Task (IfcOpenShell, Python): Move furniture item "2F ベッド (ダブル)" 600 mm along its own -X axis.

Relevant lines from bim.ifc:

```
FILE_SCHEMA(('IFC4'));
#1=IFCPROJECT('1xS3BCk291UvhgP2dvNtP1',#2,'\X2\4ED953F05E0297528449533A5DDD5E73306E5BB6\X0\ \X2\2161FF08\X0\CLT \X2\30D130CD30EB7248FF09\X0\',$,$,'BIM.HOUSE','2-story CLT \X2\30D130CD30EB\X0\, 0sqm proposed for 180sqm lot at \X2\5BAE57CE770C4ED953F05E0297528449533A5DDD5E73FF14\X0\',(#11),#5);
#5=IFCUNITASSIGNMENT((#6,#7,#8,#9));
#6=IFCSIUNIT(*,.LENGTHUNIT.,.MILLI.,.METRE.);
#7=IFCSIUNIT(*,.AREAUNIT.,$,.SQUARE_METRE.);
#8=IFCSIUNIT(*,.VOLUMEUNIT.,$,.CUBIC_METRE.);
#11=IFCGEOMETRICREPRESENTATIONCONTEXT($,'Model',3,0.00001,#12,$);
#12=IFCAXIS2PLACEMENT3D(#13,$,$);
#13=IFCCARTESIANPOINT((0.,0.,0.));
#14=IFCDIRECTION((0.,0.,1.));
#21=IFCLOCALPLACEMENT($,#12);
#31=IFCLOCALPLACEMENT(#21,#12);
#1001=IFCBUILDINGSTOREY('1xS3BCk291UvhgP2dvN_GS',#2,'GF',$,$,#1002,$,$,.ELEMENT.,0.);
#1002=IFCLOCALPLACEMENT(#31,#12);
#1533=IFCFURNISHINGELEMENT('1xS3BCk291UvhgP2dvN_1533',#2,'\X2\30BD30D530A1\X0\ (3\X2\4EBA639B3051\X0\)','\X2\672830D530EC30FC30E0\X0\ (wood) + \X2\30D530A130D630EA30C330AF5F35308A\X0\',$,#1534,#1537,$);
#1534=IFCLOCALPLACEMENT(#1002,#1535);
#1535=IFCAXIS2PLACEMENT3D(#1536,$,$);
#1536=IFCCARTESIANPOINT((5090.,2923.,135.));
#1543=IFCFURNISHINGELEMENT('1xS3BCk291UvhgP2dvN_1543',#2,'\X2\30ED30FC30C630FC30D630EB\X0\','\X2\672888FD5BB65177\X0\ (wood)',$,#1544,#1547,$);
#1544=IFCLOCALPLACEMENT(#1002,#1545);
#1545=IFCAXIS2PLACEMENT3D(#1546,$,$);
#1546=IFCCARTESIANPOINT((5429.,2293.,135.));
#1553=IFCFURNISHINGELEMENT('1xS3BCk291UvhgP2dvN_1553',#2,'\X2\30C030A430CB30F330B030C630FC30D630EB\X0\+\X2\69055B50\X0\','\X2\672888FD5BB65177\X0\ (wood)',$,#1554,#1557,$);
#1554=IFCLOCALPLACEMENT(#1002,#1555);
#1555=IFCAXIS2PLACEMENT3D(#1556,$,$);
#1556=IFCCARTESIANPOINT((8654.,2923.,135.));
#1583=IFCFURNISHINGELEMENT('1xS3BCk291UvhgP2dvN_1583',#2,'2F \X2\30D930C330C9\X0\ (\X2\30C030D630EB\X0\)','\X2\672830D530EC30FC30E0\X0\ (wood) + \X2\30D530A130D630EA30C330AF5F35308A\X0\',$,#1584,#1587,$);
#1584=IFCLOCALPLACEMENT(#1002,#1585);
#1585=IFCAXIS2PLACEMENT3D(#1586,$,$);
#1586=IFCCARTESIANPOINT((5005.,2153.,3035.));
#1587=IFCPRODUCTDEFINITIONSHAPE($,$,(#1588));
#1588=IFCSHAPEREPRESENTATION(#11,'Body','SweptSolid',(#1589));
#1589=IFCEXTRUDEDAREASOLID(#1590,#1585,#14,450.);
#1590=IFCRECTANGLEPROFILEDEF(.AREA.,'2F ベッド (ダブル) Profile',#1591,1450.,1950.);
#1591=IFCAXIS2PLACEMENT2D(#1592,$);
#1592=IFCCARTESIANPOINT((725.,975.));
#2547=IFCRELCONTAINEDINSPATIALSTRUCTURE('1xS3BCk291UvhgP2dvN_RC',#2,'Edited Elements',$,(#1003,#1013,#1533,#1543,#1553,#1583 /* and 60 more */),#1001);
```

```python
import ifcopenshell
import ifcopenshell.api.geometry
import ifcopenshell.util.placement
import ifcopenshell.util.unit

model = ifcopenshell.open("bim.ifc")
unit_scale = ifcopenshell.util.unit.calculate_unit_scale(model)

item = model.by_guid("1xS3BCk291UvhgP2dvN_1583")
matrix = ifcopenshell.util.placement.get_local_placement(item.ObjectPlacement)
matrix[:3, 3] -= matrix[:3, 0] * 0.6 / unit_scale
ifcopenshell.api.geometry.edit_object_placement(model, product=item, matrix=matrix, is_si=False)

print(ifcopenshell.util.placement.get_local_placement(item.ObjectPlacement).round(3) + 0.0)

model.write("bim-out.ifc")
```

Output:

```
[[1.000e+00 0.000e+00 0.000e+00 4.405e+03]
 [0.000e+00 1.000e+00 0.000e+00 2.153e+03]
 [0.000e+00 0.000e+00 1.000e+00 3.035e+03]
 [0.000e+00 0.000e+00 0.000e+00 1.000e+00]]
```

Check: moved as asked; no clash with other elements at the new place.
